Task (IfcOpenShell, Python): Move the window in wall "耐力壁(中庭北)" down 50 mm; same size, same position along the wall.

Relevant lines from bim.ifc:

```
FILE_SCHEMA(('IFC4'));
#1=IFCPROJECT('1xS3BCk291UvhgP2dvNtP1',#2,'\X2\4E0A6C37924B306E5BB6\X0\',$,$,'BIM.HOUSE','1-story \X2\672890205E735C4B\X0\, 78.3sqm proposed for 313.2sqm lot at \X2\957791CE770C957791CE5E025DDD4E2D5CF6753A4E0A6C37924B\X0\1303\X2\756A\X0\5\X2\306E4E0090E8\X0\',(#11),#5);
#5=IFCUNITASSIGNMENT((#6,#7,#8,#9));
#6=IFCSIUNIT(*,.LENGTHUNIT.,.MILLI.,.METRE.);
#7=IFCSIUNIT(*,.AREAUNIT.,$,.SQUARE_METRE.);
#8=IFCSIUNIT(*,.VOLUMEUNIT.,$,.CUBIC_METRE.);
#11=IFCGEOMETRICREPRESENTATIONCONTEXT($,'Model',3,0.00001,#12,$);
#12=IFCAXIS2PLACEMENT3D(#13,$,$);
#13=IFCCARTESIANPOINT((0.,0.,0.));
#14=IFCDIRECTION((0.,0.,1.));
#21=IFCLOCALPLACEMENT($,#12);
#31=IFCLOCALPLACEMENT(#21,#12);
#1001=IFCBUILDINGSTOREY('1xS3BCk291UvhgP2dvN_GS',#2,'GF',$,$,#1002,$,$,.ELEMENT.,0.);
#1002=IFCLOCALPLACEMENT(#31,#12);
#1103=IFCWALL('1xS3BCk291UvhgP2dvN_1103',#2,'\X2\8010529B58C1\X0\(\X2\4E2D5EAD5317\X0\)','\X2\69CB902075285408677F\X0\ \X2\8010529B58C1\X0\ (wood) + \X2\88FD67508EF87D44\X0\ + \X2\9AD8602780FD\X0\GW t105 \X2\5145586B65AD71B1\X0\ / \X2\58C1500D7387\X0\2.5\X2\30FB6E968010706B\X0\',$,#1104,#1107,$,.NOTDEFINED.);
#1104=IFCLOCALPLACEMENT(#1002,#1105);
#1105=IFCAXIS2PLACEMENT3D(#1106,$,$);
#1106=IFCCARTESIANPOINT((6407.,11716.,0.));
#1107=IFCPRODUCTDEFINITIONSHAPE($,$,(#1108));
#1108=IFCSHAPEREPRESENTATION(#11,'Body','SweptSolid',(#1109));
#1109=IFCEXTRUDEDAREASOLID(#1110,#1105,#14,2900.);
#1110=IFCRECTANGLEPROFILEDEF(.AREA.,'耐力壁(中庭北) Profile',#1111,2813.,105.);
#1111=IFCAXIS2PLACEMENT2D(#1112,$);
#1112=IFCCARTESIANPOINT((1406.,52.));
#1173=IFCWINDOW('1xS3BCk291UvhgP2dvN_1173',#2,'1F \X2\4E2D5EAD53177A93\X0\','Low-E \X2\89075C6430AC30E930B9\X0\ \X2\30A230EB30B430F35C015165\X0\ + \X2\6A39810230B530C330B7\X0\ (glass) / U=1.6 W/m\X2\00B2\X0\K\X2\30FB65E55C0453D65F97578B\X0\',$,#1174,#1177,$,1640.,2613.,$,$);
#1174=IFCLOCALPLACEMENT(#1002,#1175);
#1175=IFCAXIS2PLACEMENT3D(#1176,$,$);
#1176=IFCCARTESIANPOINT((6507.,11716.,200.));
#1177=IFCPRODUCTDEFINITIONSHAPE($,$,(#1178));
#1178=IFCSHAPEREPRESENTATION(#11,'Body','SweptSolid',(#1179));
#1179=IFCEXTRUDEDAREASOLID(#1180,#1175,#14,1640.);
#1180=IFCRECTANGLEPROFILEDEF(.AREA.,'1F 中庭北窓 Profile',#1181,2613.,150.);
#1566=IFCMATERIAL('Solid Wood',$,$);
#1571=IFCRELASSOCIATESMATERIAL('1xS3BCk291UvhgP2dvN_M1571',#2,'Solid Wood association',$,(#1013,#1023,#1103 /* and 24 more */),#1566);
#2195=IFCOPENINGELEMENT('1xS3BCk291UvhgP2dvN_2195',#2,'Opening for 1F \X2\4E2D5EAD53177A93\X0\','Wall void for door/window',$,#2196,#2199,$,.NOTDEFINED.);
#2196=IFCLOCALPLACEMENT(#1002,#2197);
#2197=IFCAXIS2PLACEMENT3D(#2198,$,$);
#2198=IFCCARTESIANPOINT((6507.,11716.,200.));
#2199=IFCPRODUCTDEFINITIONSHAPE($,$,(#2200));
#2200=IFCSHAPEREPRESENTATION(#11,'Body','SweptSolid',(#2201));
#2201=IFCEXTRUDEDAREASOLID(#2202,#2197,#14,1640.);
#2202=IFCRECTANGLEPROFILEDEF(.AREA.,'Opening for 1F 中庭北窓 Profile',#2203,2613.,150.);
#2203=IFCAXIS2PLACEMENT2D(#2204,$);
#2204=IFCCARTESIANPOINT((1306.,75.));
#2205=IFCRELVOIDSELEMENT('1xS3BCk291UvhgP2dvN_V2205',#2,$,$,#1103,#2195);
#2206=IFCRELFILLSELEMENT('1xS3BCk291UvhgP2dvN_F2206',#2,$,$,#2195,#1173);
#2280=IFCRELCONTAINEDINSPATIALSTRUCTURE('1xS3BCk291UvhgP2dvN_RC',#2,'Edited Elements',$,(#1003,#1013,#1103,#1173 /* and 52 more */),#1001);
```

```python
import numpy as np
import ifcopenshell
import ifcopenshell.api.geometry
import ifcopenshell.util.placement
import ifcopenshell.util.unit

model = ifcopenshell.open("bim.ifc")
unit_scale = ifcopenshell.util.unit.calculate_unit_scale(model)

window = model.by_guid("1xS3BCk291UvhgP2dvN_1173")
opening = window.FillsVoids[0].RelatingOpeningElement
dz = -0.05 / unit_scale

shift = np.array([0.0, 0.0, dz])
# The window is not placed relative to its opening, so move both.
for product in (opening, window):
    matrix = ifcopenshell.util.placement.get_local_placement(product.ObjectPlacement)
    matrix[:3, 3] += shift
    ifcopenshell.api.geometry.edit_object_placement(model, product=product, matrix=matrix, is_si=False)

print(f"moved by {dz * unit_scale:+.3f} m")

model.write("bim_edited.ifc")
```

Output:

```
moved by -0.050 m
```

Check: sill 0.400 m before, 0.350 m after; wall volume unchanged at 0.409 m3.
